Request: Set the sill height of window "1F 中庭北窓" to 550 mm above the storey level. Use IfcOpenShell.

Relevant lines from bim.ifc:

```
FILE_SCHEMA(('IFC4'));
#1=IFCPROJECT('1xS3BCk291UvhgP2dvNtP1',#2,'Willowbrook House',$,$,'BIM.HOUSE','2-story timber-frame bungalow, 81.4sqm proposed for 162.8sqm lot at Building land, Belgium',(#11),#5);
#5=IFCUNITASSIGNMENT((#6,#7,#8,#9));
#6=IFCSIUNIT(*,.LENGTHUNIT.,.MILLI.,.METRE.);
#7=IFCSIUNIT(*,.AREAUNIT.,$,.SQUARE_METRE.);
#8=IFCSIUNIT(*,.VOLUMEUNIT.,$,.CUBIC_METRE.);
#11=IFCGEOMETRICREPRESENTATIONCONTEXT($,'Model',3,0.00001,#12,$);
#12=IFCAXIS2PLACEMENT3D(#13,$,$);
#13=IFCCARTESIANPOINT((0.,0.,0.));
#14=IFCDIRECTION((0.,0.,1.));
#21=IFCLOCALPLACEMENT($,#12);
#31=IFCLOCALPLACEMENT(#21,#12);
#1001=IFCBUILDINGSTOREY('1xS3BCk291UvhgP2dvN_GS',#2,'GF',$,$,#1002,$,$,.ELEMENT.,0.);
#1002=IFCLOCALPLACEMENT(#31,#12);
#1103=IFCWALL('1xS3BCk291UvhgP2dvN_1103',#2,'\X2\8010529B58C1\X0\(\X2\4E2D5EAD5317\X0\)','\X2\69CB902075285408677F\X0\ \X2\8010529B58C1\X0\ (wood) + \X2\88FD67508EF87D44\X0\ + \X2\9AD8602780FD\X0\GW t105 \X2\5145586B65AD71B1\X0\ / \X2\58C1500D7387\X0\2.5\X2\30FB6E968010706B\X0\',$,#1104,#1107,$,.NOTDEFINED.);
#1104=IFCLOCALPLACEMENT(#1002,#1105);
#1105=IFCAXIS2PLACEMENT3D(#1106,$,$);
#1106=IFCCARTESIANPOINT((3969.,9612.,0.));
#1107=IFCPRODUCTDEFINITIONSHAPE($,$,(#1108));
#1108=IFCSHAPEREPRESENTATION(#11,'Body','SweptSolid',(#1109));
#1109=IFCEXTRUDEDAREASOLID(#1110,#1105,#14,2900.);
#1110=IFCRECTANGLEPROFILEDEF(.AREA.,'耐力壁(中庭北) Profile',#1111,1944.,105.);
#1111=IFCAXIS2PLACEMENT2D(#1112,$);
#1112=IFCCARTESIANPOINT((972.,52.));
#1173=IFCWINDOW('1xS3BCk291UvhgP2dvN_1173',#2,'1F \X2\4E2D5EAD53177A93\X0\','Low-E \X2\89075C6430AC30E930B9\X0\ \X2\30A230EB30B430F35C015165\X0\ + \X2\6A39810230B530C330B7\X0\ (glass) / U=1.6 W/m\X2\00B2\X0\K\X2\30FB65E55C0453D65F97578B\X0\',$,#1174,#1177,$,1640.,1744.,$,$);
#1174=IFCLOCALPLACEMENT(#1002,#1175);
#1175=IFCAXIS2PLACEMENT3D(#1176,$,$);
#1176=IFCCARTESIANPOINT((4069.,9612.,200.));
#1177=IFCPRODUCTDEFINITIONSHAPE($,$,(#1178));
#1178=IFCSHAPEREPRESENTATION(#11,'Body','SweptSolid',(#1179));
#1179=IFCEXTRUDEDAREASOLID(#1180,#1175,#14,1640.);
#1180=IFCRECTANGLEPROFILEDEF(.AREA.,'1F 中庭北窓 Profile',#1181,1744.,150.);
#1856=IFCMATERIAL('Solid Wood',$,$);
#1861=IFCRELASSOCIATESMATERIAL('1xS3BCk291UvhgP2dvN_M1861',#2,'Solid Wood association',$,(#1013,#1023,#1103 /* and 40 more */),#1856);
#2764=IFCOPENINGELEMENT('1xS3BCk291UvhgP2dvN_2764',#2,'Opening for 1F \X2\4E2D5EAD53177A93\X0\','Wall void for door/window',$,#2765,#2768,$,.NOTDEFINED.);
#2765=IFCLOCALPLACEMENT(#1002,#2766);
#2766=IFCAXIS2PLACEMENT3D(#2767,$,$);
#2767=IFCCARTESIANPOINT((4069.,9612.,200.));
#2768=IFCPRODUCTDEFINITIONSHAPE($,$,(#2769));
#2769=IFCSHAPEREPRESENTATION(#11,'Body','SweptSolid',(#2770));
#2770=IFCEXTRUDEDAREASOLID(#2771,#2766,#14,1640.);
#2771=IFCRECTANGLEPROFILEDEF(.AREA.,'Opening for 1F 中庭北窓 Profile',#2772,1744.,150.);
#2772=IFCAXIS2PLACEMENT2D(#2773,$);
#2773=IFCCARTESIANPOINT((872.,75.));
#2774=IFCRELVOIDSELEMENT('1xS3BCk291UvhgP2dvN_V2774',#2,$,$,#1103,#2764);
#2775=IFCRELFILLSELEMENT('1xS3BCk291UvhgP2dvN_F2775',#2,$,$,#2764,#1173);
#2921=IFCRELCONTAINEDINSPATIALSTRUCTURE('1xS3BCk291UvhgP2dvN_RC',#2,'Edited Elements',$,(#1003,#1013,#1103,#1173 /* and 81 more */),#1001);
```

```python
import numpy as np
import ifcopenshell
import ifcopenshell.api.geometry
import ifcopenshell.geom
import ifcopenshell.util.element
import ifcopenshell.util.placement
import ifcopenshell.util.shape
import ifcopenshell.util.unit

model = ifcopenshell.open("bim.ifc")
unit_scale = ifcopenshell.util.unit.calculate_unit_scale(model)

window = model.by_guid("1xS3BCk291UvhgP2dvN_1173")
opening = window.FillsVoids[0].RelatingOpeningElement
storey = ifcopenshell.util.element.get_container(window, ifc_class="IfcBuildingStorey")
level = ifcopenshell.util.placement.get_local_placement(storey.ObjectPlacement)[2, 3]

# The opening's origin need not be at the sill, so measure its lowest point.
shape = ifcopenshell.geom.create_shape(ifcopenshell.geom.settings(), opening)
bottom = ifcopenshell.util.shape.get_shape_bottom_elevation(shape, shape.geometry) / unit_scale
dz = level + 550.0 - bottom

shift = np.array([0.0, 0.0, dz])
# The window is not placed relative to its opening, so move both.
for product in (opening, window):
    matrix = ifcopenshell.util.placement.get_local_placement(product.ObjectPlacement)
    matrix[:3, 3] += shift
    ifcopenshell.api.geometry.edit_object_placement(model, product=product, matrix=matrix, is_si=False)

print(f"moved by {dz * unit_scale:+.3f} m")

model.write("bim-out.ifc")
```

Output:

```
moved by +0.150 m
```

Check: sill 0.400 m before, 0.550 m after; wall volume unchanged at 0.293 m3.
